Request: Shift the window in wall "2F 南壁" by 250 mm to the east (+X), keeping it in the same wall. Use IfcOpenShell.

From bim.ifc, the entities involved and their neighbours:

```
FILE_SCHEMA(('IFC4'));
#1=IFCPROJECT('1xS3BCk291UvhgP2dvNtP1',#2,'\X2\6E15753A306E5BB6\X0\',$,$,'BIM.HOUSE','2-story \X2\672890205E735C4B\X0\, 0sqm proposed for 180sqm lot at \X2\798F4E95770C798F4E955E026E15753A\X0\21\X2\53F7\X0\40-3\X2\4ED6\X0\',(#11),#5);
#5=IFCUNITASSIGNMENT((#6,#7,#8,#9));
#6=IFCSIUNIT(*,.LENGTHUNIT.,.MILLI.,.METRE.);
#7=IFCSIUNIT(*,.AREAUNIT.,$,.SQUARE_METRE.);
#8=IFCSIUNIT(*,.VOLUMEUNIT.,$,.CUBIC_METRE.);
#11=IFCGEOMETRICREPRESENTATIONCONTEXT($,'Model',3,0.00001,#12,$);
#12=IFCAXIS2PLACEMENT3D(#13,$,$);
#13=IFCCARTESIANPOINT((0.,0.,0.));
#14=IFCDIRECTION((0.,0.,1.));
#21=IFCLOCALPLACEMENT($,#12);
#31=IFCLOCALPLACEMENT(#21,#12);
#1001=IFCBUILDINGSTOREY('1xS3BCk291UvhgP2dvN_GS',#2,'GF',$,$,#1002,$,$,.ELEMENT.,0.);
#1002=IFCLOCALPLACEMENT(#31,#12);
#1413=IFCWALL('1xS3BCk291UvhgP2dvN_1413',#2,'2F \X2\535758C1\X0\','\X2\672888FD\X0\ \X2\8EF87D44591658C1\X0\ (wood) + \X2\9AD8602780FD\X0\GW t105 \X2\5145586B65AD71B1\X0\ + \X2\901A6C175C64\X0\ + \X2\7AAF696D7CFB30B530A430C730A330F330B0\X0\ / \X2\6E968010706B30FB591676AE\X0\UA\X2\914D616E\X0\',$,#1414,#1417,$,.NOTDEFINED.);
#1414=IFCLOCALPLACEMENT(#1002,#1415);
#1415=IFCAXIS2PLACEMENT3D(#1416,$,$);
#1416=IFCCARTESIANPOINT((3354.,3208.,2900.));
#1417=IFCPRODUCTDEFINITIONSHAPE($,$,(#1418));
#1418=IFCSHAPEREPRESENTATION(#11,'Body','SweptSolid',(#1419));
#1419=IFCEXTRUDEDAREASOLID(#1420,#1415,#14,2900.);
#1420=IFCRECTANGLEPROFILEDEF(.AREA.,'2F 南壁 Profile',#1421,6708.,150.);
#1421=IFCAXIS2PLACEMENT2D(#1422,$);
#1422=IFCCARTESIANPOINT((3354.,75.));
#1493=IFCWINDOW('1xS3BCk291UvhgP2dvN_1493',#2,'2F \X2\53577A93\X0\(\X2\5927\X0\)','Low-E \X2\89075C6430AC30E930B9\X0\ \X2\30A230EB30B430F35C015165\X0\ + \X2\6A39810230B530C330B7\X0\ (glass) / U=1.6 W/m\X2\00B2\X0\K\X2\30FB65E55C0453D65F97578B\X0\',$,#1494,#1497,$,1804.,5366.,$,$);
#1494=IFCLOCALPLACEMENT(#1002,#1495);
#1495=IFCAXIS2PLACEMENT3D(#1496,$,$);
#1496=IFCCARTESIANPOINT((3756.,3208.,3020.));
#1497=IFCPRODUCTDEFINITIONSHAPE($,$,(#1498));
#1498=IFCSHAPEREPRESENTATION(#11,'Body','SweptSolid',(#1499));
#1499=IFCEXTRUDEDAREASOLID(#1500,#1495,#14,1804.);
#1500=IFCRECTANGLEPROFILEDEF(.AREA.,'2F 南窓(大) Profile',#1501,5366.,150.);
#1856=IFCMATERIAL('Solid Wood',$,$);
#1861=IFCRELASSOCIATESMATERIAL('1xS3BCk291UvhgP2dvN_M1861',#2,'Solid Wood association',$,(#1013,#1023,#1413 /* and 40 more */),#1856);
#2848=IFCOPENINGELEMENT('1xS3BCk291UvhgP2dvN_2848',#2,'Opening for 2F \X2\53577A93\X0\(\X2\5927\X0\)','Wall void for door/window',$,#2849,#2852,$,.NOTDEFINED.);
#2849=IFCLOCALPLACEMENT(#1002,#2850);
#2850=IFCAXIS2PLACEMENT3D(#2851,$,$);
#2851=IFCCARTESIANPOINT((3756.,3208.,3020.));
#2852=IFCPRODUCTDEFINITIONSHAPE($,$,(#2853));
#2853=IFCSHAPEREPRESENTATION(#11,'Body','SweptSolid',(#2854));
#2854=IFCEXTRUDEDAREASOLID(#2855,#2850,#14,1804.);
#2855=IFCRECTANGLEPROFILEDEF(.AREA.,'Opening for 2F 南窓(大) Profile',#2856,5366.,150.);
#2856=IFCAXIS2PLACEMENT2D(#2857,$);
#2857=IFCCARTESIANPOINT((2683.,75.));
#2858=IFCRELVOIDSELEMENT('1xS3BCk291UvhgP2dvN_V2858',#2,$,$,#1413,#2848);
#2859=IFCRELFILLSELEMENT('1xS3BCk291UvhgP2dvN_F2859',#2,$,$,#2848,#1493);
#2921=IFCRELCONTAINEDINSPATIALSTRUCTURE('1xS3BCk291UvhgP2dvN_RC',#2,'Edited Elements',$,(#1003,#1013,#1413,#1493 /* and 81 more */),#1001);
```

```python
import ifcopenshell
import ifcopenshell.api.geometry
import ifcopenshell.util.placement

model = ifcopenshell.open("bim.ifc")

window = model.by_guid("1xS3BCk291UvhgP2dvN_1493")
opening = window.FillsVoids[0].RelatingOpeningElement
wall = opening.VoidsElements[0].RelatingBuildingElement

wall_matrix = ifcopenshell.util.placement.get_local_placement(wall.ObjectPlacement)
shift = wall_matrix[:3, 0] * 250.0
before = ifcopenshell.util.placement.get_local_placement(window.ObjectPlacement)[:3, 3].copy()

# The window is not placed relative to its opening, so move both.
for product in (opening, window):
    matrix = ifcopenshell.util.placement.get_local_placement(product.ObjectPlacement)
    matrix[:3, 3] += shift
    ifcopenshell.api.geometry.edit_object_placement(model, product=product, matrix=matrix, is_si=False)

after = ifcopenshell.util.placement.get_local_placement(window.ObjectPlacement)[:3, 3]
print("window moved by", (after - before).round(3) + 0.0)

model.write("bim_v2.ifc")
```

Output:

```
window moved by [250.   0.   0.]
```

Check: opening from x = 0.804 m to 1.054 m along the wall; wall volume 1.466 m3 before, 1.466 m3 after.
